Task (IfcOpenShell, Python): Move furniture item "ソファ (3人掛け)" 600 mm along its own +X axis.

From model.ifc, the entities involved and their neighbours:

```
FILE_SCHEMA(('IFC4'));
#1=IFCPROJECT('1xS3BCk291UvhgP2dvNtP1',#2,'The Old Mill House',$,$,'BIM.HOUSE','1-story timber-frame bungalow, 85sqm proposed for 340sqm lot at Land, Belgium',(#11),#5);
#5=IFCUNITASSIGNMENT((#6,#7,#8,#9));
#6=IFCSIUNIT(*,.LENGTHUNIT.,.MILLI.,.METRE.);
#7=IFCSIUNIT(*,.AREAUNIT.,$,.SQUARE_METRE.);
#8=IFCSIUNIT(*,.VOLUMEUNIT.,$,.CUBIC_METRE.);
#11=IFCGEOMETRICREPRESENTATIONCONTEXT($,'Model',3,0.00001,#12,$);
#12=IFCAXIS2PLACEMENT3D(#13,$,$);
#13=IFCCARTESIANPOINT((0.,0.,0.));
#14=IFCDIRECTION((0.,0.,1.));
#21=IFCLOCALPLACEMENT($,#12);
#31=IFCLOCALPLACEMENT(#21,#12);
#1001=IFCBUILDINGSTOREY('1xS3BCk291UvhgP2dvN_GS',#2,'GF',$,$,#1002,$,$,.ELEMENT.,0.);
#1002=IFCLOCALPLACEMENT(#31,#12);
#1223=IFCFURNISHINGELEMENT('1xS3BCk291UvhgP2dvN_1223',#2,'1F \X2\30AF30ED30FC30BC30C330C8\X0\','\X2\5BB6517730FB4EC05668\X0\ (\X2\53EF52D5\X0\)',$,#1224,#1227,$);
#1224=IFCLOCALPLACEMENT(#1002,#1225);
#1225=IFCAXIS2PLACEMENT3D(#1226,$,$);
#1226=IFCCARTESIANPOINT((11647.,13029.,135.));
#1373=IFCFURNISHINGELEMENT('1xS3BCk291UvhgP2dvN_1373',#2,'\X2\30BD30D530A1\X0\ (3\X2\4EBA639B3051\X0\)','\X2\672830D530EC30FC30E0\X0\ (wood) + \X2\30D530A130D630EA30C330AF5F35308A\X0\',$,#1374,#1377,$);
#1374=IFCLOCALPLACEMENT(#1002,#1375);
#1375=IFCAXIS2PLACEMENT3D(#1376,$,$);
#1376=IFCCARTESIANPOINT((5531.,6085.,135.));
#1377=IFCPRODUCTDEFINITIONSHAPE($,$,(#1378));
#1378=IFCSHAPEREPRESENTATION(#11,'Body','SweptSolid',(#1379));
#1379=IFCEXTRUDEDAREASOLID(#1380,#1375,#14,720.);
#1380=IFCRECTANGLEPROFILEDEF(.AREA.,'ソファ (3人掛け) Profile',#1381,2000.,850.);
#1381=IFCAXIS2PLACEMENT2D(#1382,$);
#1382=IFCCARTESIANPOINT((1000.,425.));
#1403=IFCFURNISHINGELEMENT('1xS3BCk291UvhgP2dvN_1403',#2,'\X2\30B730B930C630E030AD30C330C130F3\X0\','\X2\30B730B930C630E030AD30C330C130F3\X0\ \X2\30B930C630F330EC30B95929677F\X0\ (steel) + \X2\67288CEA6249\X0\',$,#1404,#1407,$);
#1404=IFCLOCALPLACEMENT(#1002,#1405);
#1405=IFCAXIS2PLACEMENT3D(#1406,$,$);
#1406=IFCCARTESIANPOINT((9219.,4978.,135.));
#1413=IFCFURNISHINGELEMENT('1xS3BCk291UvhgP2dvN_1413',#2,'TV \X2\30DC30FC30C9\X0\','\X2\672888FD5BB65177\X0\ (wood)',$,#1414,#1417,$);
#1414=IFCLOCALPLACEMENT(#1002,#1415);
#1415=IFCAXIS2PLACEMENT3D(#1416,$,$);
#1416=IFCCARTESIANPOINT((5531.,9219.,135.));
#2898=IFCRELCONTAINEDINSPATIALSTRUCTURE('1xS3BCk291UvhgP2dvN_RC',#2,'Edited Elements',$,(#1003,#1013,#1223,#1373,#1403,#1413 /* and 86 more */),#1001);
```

```python
import ifcopenshell
import ifcopenshell.api.geometry
import ifcopenshell.util.placement

model = ifcopenshell.open("model.ifc")

item = model.by_id(1373)
matrix = ifcopenshell.util.placement.get_local_placement(item.ObjectPlacement)
matrix[:3, 3] += matrix[:3, 0] * 600.0
ifcopenshell.api.geometry.edit_object_placement(model, product=item, matrix=matrix, is_si=False)

print(ifcopenshell.util.placement.get_local_placement(item.ObjectPlacement).round(3) + 0.0)

model.write("model_updated.ifc")
```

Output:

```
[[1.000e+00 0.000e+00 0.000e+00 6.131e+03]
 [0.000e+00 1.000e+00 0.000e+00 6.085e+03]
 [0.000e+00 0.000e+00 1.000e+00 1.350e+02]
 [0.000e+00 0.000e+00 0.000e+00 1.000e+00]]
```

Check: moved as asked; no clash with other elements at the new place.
